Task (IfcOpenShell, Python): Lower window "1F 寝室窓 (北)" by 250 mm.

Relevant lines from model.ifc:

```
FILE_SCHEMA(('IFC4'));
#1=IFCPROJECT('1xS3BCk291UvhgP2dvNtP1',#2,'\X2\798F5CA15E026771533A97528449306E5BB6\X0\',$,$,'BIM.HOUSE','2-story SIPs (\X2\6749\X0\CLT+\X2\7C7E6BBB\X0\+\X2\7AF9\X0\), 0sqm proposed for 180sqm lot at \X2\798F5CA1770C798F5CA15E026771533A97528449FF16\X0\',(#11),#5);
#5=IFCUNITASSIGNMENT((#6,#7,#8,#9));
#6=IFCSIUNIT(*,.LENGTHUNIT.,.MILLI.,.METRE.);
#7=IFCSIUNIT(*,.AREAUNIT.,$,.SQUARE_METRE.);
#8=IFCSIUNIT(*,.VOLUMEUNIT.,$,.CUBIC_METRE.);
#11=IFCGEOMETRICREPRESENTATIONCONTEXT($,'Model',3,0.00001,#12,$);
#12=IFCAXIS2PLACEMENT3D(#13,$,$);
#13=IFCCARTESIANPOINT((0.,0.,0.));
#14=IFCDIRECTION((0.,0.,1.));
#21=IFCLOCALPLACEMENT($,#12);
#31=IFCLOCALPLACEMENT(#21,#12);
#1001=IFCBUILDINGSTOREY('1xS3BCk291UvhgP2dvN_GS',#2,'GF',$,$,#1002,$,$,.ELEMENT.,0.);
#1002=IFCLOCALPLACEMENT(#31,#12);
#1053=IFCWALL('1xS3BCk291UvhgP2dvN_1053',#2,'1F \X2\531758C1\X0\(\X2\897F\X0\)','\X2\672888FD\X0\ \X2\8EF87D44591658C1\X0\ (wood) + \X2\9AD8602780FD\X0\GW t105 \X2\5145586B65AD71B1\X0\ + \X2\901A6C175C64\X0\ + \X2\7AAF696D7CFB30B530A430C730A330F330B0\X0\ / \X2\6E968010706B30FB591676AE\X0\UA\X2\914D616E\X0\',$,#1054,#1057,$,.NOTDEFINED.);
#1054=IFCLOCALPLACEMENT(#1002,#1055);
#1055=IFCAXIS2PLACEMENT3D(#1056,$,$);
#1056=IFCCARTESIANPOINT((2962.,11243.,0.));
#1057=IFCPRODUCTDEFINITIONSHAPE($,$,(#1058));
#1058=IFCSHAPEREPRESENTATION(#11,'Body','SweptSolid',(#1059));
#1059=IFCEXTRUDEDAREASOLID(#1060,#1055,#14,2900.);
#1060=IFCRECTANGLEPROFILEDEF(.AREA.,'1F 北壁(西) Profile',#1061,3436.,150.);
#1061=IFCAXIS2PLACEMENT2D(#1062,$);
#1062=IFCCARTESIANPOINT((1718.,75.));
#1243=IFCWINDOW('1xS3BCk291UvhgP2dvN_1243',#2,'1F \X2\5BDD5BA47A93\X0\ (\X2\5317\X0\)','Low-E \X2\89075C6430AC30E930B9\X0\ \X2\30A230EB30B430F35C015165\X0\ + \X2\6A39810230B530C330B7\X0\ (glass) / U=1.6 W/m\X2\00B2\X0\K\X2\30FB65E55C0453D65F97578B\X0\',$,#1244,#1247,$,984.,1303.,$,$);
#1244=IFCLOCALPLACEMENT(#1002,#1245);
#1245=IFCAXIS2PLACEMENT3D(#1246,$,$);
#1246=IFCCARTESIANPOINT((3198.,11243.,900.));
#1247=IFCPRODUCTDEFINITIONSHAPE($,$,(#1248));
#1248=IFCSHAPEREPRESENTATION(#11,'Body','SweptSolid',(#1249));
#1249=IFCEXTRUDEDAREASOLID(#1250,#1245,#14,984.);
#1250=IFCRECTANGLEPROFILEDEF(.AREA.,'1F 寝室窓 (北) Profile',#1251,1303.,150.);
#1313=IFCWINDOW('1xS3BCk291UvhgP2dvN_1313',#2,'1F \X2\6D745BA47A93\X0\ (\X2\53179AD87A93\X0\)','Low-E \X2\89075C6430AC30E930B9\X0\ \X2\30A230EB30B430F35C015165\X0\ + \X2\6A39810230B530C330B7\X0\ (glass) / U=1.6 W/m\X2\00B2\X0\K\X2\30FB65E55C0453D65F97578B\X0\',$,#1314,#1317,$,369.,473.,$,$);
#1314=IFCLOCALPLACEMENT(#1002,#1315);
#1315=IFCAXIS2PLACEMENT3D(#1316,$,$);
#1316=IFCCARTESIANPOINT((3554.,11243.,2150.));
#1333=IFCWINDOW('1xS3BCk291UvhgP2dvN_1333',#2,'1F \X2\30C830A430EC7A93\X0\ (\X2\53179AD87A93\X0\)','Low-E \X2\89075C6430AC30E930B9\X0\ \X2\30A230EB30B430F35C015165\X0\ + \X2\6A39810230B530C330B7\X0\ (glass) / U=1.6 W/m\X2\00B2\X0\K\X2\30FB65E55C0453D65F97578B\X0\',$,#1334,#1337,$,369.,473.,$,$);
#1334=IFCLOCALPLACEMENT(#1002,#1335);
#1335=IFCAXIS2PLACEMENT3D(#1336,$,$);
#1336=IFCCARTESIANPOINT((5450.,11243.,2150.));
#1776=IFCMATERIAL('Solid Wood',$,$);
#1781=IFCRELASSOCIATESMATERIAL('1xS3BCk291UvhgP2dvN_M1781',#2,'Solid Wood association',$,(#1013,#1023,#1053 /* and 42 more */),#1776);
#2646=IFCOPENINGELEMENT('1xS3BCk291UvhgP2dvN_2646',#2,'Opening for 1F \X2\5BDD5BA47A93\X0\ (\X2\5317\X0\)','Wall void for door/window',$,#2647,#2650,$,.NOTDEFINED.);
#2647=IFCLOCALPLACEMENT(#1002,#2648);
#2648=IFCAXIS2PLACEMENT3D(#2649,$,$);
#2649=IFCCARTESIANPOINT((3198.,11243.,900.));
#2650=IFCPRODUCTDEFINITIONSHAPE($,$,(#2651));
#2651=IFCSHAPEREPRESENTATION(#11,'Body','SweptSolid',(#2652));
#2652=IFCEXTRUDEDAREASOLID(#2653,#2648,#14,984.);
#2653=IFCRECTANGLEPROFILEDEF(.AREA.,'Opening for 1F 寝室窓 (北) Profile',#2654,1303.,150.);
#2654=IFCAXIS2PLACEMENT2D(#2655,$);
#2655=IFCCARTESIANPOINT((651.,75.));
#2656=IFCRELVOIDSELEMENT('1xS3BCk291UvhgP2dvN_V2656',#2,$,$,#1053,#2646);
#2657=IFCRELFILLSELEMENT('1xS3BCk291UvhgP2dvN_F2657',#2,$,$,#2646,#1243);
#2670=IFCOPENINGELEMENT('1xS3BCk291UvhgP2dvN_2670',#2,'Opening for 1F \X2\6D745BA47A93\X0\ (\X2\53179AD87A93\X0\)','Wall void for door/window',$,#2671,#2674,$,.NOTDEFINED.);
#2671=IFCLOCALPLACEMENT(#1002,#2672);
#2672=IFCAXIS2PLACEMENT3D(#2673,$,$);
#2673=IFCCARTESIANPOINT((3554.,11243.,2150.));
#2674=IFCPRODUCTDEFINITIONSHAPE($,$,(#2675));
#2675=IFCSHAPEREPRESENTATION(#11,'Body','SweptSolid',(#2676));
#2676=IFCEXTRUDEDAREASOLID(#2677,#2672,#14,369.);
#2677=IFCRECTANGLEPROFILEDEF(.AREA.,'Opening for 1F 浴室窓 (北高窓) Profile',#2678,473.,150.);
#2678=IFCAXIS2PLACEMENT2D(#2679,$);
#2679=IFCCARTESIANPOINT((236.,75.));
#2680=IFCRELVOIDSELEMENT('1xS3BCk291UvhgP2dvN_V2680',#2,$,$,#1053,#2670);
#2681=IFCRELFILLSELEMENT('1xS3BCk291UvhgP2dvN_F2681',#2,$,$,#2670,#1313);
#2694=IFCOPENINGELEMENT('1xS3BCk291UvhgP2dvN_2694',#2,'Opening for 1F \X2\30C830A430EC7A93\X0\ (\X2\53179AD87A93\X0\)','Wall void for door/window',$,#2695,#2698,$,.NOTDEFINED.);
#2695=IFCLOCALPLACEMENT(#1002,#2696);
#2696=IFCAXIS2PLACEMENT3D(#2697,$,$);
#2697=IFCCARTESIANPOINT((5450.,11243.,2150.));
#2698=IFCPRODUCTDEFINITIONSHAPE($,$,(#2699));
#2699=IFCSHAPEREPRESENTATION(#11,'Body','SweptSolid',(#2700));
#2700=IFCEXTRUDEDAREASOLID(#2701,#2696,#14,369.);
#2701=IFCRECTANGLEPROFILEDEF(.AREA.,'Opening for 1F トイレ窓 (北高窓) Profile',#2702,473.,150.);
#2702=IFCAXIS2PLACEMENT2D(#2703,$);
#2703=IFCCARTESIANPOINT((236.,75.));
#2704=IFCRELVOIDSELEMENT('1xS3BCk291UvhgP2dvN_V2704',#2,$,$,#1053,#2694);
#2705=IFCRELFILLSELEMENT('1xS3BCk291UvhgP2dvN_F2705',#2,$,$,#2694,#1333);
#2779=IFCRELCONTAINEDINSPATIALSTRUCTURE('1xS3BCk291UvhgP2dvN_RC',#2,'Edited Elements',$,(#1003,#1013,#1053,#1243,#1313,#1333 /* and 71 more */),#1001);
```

```python
import numpy as np
import ifcopenshell
import ifcopenshell.api.geometry
import ifcopenshell.util.placement
import ifcopenshell.util.unit

model = ifcopenshell.open("model.ifc")
unit_scale = ifcopenshell.util.unit.calculate_unit_scale(model)

window = model.by_guid("1xS3BCk291UvhgP2dvN_1243")
opening = window.FillsVoids[0].RelatingOpeningElement
dz = -0.25 / unit_scale

shift = np.array([0.0, 0.0, dz])
# The window is not placed relative to its opening, so move both.
for product in (opening, window):
    matrix = ifcopenshell.util.placement.get_local_placement(product.ObjectPlacement)
    matrix[:3, 3] += shift
    ifcopenshell.api.geometry.edit_object_placement(model, product=product, matrix=matrix, is_si=False)

print(f"moved by {dz * unit_scale:+.3f} m")

model.write("model_edited.ifc")
```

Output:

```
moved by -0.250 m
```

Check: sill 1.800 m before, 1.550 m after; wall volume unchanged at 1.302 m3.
